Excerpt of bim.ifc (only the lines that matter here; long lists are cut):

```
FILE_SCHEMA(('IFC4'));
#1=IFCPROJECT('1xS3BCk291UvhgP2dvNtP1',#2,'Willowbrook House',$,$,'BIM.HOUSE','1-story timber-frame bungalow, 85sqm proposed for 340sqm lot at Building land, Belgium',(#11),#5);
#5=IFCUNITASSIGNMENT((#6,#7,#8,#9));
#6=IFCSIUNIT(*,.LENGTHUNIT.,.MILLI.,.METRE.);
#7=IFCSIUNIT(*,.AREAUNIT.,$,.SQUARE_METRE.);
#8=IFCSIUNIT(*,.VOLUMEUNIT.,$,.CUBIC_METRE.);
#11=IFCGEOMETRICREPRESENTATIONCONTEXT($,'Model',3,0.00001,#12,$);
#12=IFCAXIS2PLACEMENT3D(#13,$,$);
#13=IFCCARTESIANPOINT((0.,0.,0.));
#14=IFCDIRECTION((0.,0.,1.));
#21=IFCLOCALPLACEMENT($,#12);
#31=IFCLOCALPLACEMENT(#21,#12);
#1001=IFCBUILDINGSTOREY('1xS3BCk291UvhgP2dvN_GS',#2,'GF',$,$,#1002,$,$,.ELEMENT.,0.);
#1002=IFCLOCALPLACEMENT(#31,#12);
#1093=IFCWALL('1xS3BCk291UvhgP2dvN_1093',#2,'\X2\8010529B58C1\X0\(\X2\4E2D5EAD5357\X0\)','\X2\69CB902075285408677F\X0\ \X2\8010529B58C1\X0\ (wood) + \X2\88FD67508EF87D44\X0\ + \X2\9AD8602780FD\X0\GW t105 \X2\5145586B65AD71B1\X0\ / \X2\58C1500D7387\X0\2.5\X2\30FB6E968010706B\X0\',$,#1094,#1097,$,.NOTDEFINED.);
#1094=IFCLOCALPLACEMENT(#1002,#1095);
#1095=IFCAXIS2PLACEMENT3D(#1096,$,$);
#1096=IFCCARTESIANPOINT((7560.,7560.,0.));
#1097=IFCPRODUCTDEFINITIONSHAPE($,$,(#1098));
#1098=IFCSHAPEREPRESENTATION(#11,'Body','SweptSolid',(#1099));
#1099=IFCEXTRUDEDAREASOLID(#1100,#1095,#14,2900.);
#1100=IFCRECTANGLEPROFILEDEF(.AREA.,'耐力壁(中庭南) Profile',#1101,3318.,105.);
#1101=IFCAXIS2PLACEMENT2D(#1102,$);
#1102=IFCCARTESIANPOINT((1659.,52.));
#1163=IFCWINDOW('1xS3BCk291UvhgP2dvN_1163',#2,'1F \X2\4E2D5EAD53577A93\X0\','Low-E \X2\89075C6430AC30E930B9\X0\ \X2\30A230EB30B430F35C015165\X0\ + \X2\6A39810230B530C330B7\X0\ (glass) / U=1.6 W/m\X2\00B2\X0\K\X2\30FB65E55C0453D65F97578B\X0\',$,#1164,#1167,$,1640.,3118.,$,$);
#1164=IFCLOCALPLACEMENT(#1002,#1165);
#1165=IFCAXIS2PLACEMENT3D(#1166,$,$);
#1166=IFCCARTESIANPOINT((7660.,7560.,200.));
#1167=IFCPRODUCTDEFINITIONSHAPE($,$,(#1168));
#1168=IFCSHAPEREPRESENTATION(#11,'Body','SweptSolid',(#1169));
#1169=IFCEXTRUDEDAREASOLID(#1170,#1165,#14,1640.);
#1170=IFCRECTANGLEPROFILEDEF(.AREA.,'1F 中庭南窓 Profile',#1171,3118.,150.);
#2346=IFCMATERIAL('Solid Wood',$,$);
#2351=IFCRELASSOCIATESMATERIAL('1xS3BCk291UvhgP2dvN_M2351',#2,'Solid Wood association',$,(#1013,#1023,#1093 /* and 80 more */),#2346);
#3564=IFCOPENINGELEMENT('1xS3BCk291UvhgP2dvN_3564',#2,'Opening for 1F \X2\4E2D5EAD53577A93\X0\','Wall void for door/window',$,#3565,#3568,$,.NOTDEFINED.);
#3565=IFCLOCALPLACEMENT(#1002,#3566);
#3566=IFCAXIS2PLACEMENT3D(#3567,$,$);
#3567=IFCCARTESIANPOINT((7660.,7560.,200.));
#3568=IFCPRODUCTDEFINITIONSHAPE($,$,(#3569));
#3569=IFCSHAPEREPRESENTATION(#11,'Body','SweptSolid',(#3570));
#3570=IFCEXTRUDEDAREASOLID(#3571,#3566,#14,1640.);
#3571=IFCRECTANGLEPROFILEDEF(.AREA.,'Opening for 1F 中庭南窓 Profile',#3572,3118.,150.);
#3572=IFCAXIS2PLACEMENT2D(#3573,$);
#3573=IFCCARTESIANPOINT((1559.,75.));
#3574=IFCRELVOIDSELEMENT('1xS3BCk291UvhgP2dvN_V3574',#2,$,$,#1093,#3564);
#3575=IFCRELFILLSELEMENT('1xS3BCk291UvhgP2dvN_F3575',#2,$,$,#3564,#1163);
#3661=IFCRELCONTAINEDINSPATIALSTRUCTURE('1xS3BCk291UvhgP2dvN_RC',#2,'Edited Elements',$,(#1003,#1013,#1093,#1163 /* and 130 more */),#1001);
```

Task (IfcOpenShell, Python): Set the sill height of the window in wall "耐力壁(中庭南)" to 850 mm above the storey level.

```python
import numpy as np
import ifcopenshell
import ifcopenshell.api.geometry
import ifcopenshell.geom
import ifcopenshell.util.element
import ifcopenshell.util.placement
import ifcopenshell.util.shape
import ifcopenshell.util.unit

model = ifcopenshell.open("bim.ifc")
unit_scale = ifcopenshell.util.unit.calculate_unit_scale(model)

window = model.by_guid("1xS3BCk291UvhgP2dvN_1163")
opening = window.FillsVoids[0].RelatingOpeningElement
storey = ifcopenshell.util.element.get_container(window, ifc_class="IfcBuildingStorey")
level = ifcopenshell.util.placement.get_local_placement(storey.ObjectPlacement)[2, 3]

# The opening's origin need not be at the sill, so measure its lowest point.
shape = ifcopenshell.geom.create_shape(ifcopenshell.geom.settings(), opening)
bottom = ifcopenshell.util.shape.get_shape_bottom_elevation(shape, shape.geometry) / unit_scale
dz = level + 850.0 - bottom

shift = np.array([0.0, 0.0, dz])
# The window is not placed relative to its opening, so move both.
for product in (opening, window):
    matrix = ifcopenshell.util.placement.get_local_placement(product.ObjectPlacement)
    matrix[:3, 3] += shift
    ifcopenshell.api.geometry.edit_object_placement(model, product=product, matrix=matrix, is_si=False)

print(f"moved by {dz * unit_scale:+.3f} m")

model.write("bim-out.ifc")
```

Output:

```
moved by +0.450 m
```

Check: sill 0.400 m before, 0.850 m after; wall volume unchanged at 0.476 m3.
